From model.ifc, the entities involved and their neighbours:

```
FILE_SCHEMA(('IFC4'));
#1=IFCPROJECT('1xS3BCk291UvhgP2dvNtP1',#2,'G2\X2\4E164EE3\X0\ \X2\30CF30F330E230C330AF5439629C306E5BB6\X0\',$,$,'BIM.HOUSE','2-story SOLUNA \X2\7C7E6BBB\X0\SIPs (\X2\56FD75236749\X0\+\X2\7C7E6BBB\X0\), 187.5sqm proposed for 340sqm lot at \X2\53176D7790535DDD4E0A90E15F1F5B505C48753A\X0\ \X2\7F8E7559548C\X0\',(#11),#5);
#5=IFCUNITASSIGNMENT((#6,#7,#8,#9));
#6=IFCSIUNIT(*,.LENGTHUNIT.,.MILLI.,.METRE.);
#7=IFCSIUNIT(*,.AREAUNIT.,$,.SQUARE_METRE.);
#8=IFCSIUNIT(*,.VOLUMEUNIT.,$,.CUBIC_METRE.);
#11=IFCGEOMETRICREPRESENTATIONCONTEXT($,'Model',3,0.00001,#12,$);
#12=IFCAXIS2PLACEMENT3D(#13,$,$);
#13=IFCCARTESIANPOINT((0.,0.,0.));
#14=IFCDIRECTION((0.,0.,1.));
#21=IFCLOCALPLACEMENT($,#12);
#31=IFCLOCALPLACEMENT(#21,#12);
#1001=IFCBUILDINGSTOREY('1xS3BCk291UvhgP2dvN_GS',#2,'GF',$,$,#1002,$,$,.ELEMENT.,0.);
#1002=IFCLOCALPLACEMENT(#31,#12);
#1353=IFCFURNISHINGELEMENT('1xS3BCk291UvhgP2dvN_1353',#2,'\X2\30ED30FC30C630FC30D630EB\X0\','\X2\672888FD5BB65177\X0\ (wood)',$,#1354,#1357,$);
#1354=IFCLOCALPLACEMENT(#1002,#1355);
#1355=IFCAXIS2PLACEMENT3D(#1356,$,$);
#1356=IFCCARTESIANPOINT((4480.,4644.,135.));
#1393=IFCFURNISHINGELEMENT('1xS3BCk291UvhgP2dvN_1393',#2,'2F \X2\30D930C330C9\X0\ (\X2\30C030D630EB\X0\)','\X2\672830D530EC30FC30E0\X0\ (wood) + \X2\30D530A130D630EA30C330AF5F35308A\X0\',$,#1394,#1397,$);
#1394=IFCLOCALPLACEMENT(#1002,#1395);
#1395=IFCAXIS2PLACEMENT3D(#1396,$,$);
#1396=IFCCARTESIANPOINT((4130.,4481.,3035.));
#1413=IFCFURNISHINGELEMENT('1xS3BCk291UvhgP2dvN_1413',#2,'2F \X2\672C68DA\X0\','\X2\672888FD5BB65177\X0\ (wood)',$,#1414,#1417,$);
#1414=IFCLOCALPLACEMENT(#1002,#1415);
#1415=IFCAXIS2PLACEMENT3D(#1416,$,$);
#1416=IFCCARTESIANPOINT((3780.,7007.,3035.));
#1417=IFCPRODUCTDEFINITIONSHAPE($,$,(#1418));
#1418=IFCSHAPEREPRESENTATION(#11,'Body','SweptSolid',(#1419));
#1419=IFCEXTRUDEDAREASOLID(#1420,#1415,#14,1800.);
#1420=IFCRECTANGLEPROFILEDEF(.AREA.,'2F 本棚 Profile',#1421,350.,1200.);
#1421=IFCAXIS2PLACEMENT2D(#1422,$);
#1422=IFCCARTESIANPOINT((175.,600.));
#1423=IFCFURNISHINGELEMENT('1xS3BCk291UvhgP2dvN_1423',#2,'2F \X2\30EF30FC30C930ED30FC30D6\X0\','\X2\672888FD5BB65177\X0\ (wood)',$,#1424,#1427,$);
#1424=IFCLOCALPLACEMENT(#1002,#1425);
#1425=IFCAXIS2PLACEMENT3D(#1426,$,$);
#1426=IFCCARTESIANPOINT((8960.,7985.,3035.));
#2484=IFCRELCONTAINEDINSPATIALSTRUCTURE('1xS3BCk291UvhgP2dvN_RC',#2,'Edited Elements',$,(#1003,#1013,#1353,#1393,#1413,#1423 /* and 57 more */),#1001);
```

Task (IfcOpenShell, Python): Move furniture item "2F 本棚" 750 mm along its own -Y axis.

```python
import ifcopenshell
import ifcopenshell.api.geometry
import ifcopenshell.util.placement
import ifcopenshell.util.unit

model = ifcopenshell.open("model.ifc")
unit_scale = ifcopenshell.util.unit.calculate_unit_scale(model)

item = model.by_guid("1xS3BCk291UvhgP2dvN_1413")
matrix = ifcopenshell.util.placement.get_local_placement(item.ObjectPlacement)
matrix[:3, 3] -= matrix[:3, 1] * 0.75 / unit_scale
ifcopenshell.api.geometry.edit_object_placement(model, product=item, matrix=matrix, is_si=False)

print(ifcopenshell.util.placement.get_local_placement(item.ObjectPlacement).round(3) + 0.0)

model.write("model_rev.ifc")
```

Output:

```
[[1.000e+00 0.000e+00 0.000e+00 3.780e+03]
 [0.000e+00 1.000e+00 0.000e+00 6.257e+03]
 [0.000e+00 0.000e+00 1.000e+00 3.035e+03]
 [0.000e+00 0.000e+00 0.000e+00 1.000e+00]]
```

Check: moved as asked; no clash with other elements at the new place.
